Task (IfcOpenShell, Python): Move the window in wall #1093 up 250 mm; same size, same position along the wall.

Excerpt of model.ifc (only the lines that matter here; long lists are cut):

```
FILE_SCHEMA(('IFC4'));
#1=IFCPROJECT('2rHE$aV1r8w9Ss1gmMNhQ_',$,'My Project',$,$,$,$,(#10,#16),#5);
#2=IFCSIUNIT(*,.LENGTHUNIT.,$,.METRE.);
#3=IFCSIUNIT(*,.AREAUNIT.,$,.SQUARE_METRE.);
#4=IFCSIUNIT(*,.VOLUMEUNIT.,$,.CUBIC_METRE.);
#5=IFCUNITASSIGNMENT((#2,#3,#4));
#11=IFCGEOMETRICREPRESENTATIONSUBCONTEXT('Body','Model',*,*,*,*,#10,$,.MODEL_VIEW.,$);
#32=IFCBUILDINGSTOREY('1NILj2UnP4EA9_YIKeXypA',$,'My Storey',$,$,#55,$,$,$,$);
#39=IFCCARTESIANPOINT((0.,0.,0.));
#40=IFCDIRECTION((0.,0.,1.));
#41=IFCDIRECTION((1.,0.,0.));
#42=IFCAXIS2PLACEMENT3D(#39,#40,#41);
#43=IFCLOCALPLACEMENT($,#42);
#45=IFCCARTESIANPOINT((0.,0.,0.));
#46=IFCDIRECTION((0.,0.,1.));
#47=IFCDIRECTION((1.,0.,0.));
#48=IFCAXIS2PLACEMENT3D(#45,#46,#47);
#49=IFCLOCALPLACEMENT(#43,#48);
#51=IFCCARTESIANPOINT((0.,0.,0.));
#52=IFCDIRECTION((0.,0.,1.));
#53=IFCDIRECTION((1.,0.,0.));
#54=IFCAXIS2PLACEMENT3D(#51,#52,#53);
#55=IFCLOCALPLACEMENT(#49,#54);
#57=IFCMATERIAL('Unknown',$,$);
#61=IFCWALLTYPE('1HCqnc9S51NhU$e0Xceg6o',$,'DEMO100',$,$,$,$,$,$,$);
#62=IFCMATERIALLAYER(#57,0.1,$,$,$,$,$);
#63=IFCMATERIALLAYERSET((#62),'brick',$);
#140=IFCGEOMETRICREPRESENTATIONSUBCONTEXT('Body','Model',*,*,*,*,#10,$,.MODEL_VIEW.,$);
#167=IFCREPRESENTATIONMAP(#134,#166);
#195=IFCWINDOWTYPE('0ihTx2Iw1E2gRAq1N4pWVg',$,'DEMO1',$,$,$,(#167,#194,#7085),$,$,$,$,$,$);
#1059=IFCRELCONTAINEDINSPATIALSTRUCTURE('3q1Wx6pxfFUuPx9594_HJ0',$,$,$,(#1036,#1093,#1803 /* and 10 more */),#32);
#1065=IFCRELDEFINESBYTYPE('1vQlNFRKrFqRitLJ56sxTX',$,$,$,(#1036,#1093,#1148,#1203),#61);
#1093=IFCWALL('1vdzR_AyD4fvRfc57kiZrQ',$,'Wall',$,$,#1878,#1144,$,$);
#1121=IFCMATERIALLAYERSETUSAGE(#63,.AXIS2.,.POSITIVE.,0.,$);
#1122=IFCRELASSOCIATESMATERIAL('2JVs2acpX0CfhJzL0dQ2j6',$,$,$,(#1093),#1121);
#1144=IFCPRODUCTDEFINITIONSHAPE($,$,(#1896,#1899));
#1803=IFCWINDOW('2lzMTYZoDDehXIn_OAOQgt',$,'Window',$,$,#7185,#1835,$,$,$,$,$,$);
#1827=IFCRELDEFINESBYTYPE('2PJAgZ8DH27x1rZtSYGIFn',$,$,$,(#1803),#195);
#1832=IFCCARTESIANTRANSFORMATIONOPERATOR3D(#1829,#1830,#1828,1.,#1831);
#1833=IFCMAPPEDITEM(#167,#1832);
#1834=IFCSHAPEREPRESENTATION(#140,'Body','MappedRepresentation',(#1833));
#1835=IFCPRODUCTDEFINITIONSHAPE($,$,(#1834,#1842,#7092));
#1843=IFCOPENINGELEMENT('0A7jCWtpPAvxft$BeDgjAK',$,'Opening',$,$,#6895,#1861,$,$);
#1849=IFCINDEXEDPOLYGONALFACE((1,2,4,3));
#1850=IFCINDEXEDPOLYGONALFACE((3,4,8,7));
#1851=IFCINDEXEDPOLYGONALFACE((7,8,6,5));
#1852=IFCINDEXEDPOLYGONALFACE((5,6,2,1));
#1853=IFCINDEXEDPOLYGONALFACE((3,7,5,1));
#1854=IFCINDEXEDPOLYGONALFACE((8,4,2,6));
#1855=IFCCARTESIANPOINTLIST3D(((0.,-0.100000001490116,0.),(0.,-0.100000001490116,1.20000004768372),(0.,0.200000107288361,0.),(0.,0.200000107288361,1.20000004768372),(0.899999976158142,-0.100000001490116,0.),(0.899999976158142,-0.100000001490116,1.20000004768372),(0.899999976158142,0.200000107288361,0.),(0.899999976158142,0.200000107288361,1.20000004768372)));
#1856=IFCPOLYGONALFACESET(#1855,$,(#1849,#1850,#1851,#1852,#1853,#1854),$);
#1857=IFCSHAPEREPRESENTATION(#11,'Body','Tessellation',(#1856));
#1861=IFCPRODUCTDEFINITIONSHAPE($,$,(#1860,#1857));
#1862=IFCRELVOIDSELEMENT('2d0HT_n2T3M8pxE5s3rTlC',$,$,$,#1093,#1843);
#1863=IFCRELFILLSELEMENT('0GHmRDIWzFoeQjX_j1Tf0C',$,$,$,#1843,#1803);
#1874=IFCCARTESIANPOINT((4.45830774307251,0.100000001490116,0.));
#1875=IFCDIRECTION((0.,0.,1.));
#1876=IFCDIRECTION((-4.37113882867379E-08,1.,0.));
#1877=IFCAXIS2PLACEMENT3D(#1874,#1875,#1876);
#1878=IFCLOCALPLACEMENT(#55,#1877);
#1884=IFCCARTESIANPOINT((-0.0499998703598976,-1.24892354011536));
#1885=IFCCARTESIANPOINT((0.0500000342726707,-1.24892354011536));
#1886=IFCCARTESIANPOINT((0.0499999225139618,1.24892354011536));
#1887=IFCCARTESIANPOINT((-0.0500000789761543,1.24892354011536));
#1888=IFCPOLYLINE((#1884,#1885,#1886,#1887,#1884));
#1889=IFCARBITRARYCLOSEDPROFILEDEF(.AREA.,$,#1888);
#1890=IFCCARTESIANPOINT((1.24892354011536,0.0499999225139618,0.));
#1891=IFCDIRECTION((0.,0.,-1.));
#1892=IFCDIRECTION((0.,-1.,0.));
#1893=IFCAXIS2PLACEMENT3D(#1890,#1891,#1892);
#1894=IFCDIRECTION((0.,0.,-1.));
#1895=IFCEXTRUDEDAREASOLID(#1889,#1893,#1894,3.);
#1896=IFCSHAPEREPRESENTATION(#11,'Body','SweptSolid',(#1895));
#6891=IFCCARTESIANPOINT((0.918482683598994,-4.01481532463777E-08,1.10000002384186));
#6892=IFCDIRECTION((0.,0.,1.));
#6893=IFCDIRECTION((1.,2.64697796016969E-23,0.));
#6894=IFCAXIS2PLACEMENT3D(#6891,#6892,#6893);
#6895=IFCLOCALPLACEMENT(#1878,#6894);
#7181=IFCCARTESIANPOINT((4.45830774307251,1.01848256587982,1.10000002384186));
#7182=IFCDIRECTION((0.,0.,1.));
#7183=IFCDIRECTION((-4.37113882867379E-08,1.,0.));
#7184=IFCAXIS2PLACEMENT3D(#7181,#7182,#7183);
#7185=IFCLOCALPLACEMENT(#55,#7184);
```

```python
import numpy as np
import ifcopenshell
import ifcopenshell.api.geometry
import ifcopenshell.util.placement
import ifcopenshell.util.unit

model = ifcopenshell.open("model.ifc")
unit_scale = ifcopenshell.util.unit.calculate_unit_scale(model)

window = model.by_guid("2lzMTYZoDDehXIn_OAOQgt")
opening = window.FillsVoids[0].RelatingOpeningElement
dz = 0.25

shift = np.array([0.0, 0.0, dz])
# The window is not placed relative to its opening, so move both.
for product in (opening, window):
    matrix = ifcopenshell.util.placement.get_local_placement(product.ObjectPlacement)
    matrix[:3, 3] += shift
    ifcopenshell.api.geometry.edit_object_placement(model, product=product, matrix=matrix, is_si=False)

print(f"moved by {dz * unit_scale:+.3f} m")

model.write("model_rev.ifc")
```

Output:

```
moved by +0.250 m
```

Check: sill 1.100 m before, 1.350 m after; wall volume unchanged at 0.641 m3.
